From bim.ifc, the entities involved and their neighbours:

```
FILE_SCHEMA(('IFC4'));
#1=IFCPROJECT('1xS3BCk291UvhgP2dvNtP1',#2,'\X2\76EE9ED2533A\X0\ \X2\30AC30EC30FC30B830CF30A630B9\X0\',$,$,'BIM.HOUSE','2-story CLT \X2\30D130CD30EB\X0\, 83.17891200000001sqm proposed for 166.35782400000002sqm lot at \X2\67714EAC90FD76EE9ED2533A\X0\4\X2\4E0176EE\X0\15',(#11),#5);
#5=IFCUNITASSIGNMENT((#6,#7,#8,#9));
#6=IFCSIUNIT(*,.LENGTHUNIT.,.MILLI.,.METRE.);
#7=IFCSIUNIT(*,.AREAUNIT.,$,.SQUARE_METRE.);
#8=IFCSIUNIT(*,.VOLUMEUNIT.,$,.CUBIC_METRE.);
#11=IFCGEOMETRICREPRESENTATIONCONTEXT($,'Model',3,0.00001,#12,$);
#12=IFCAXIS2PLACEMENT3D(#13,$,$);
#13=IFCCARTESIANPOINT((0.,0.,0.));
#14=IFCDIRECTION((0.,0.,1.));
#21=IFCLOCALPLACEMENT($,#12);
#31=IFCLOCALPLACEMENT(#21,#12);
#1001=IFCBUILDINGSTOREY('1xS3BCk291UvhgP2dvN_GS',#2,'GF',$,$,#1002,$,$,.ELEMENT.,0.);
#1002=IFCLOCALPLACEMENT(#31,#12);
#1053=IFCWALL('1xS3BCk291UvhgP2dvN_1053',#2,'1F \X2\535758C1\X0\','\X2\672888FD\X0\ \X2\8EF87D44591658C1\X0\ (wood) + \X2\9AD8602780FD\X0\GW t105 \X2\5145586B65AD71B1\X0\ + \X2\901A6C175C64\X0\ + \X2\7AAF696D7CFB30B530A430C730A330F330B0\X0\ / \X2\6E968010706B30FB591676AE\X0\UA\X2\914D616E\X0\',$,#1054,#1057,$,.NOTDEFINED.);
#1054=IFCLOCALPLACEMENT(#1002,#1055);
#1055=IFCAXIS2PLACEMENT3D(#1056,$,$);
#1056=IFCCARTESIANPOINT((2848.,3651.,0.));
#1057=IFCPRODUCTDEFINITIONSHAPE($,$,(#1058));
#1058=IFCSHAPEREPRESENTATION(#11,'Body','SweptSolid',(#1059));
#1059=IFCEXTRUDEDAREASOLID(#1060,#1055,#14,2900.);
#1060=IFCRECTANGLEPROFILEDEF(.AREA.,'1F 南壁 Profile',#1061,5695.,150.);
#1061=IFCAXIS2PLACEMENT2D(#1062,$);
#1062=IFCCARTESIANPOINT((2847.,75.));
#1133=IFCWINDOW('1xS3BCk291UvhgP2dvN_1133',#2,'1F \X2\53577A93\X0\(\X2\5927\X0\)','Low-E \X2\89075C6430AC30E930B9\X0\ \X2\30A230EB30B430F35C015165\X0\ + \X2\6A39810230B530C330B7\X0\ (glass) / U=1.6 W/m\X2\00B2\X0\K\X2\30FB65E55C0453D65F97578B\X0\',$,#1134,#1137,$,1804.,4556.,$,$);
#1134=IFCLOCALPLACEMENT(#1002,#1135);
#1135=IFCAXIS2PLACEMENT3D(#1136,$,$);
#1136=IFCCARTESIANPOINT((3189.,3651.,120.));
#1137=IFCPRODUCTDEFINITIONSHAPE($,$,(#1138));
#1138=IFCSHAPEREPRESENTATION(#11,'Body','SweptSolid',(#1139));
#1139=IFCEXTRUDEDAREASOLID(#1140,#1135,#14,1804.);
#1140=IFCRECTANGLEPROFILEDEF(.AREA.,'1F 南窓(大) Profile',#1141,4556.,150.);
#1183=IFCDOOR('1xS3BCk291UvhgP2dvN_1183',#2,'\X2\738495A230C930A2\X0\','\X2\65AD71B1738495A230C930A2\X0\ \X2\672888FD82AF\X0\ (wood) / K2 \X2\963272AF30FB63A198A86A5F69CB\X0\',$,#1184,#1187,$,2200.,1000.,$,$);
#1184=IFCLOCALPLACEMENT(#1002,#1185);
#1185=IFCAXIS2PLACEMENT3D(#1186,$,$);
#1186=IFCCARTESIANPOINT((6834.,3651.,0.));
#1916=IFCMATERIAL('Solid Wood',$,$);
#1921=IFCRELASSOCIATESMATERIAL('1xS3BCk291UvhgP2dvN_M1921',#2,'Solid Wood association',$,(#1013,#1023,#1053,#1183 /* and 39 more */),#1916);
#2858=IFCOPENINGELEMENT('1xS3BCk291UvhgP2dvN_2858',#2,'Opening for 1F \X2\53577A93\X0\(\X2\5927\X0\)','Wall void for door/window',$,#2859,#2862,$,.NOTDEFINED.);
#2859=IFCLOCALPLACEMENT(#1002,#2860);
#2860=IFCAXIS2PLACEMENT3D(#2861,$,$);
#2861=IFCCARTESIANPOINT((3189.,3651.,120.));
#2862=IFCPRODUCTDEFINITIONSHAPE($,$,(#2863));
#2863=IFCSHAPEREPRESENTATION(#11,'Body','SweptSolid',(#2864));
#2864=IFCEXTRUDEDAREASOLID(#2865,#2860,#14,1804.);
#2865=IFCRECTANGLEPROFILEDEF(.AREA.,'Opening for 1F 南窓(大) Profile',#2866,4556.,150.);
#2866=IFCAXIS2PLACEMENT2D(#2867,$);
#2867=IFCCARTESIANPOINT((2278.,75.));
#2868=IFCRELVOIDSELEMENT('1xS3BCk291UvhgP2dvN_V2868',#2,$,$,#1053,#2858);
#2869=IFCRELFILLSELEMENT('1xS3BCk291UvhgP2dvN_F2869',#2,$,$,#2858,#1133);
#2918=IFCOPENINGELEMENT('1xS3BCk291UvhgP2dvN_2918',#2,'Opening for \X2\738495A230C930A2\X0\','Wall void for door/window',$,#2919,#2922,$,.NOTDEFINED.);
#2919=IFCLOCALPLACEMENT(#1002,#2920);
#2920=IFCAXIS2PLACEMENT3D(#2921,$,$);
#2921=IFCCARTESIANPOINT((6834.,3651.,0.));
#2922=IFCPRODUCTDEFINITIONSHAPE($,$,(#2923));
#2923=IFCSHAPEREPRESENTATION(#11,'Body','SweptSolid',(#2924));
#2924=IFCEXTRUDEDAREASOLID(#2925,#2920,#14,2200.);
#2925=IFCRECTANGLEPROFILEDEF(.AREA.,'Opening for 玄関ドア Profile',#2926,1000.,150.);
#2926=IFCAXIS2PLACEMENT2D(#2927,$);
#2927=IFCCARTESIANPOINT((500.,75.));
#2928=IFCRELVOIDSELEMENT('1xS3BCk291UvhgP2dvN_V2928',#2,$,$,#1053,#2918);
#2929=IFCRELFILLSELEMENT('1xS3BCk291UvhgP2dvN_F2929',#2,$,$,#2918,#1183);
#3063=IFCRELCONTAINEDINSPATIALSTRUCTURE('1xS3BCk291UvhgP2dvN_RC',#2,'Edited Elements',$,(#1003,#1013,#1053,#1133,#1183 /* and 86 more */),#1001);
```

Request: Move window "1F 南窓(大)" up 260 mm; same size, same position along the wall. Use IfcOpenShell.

```python
import numpy as np
import ifcopenshell
import ifcopenshell.api.geometry
import ifcopenshell.util.placement
import ifcopenshell.util.unit

model = ifcopenshell.open("bim.ifc")
unit_scale = ifcopenshell.util.unit.calculate_unit_scale(model)

window = model.by_guid("1xS3BCk291UvhgP2dvN_1133")
opening = window.FillsVoids[0].RelatingOpeningElement
dz = 0.26 / unit_scale

shift = np.array([0.0, 0.0, dz])
# The window is not placed relative to its opening, so move both.
for product in (opening, window):
    matrix = ifcopenshell.util.placement.get_local_placement(product.ObjectPlacement)
    matrix[:3, 3] += shift
    ifcopenshell.api.geometry.edit_object_placement(model, product=product, matrix=matrix, is_si=False)

print(f"moved by {dz * unit_scale:+.3f} m")

model.write("bim_rev.ifc")
```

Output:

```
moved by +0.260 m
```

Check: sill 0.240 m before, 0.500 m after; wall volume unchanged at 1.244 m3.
